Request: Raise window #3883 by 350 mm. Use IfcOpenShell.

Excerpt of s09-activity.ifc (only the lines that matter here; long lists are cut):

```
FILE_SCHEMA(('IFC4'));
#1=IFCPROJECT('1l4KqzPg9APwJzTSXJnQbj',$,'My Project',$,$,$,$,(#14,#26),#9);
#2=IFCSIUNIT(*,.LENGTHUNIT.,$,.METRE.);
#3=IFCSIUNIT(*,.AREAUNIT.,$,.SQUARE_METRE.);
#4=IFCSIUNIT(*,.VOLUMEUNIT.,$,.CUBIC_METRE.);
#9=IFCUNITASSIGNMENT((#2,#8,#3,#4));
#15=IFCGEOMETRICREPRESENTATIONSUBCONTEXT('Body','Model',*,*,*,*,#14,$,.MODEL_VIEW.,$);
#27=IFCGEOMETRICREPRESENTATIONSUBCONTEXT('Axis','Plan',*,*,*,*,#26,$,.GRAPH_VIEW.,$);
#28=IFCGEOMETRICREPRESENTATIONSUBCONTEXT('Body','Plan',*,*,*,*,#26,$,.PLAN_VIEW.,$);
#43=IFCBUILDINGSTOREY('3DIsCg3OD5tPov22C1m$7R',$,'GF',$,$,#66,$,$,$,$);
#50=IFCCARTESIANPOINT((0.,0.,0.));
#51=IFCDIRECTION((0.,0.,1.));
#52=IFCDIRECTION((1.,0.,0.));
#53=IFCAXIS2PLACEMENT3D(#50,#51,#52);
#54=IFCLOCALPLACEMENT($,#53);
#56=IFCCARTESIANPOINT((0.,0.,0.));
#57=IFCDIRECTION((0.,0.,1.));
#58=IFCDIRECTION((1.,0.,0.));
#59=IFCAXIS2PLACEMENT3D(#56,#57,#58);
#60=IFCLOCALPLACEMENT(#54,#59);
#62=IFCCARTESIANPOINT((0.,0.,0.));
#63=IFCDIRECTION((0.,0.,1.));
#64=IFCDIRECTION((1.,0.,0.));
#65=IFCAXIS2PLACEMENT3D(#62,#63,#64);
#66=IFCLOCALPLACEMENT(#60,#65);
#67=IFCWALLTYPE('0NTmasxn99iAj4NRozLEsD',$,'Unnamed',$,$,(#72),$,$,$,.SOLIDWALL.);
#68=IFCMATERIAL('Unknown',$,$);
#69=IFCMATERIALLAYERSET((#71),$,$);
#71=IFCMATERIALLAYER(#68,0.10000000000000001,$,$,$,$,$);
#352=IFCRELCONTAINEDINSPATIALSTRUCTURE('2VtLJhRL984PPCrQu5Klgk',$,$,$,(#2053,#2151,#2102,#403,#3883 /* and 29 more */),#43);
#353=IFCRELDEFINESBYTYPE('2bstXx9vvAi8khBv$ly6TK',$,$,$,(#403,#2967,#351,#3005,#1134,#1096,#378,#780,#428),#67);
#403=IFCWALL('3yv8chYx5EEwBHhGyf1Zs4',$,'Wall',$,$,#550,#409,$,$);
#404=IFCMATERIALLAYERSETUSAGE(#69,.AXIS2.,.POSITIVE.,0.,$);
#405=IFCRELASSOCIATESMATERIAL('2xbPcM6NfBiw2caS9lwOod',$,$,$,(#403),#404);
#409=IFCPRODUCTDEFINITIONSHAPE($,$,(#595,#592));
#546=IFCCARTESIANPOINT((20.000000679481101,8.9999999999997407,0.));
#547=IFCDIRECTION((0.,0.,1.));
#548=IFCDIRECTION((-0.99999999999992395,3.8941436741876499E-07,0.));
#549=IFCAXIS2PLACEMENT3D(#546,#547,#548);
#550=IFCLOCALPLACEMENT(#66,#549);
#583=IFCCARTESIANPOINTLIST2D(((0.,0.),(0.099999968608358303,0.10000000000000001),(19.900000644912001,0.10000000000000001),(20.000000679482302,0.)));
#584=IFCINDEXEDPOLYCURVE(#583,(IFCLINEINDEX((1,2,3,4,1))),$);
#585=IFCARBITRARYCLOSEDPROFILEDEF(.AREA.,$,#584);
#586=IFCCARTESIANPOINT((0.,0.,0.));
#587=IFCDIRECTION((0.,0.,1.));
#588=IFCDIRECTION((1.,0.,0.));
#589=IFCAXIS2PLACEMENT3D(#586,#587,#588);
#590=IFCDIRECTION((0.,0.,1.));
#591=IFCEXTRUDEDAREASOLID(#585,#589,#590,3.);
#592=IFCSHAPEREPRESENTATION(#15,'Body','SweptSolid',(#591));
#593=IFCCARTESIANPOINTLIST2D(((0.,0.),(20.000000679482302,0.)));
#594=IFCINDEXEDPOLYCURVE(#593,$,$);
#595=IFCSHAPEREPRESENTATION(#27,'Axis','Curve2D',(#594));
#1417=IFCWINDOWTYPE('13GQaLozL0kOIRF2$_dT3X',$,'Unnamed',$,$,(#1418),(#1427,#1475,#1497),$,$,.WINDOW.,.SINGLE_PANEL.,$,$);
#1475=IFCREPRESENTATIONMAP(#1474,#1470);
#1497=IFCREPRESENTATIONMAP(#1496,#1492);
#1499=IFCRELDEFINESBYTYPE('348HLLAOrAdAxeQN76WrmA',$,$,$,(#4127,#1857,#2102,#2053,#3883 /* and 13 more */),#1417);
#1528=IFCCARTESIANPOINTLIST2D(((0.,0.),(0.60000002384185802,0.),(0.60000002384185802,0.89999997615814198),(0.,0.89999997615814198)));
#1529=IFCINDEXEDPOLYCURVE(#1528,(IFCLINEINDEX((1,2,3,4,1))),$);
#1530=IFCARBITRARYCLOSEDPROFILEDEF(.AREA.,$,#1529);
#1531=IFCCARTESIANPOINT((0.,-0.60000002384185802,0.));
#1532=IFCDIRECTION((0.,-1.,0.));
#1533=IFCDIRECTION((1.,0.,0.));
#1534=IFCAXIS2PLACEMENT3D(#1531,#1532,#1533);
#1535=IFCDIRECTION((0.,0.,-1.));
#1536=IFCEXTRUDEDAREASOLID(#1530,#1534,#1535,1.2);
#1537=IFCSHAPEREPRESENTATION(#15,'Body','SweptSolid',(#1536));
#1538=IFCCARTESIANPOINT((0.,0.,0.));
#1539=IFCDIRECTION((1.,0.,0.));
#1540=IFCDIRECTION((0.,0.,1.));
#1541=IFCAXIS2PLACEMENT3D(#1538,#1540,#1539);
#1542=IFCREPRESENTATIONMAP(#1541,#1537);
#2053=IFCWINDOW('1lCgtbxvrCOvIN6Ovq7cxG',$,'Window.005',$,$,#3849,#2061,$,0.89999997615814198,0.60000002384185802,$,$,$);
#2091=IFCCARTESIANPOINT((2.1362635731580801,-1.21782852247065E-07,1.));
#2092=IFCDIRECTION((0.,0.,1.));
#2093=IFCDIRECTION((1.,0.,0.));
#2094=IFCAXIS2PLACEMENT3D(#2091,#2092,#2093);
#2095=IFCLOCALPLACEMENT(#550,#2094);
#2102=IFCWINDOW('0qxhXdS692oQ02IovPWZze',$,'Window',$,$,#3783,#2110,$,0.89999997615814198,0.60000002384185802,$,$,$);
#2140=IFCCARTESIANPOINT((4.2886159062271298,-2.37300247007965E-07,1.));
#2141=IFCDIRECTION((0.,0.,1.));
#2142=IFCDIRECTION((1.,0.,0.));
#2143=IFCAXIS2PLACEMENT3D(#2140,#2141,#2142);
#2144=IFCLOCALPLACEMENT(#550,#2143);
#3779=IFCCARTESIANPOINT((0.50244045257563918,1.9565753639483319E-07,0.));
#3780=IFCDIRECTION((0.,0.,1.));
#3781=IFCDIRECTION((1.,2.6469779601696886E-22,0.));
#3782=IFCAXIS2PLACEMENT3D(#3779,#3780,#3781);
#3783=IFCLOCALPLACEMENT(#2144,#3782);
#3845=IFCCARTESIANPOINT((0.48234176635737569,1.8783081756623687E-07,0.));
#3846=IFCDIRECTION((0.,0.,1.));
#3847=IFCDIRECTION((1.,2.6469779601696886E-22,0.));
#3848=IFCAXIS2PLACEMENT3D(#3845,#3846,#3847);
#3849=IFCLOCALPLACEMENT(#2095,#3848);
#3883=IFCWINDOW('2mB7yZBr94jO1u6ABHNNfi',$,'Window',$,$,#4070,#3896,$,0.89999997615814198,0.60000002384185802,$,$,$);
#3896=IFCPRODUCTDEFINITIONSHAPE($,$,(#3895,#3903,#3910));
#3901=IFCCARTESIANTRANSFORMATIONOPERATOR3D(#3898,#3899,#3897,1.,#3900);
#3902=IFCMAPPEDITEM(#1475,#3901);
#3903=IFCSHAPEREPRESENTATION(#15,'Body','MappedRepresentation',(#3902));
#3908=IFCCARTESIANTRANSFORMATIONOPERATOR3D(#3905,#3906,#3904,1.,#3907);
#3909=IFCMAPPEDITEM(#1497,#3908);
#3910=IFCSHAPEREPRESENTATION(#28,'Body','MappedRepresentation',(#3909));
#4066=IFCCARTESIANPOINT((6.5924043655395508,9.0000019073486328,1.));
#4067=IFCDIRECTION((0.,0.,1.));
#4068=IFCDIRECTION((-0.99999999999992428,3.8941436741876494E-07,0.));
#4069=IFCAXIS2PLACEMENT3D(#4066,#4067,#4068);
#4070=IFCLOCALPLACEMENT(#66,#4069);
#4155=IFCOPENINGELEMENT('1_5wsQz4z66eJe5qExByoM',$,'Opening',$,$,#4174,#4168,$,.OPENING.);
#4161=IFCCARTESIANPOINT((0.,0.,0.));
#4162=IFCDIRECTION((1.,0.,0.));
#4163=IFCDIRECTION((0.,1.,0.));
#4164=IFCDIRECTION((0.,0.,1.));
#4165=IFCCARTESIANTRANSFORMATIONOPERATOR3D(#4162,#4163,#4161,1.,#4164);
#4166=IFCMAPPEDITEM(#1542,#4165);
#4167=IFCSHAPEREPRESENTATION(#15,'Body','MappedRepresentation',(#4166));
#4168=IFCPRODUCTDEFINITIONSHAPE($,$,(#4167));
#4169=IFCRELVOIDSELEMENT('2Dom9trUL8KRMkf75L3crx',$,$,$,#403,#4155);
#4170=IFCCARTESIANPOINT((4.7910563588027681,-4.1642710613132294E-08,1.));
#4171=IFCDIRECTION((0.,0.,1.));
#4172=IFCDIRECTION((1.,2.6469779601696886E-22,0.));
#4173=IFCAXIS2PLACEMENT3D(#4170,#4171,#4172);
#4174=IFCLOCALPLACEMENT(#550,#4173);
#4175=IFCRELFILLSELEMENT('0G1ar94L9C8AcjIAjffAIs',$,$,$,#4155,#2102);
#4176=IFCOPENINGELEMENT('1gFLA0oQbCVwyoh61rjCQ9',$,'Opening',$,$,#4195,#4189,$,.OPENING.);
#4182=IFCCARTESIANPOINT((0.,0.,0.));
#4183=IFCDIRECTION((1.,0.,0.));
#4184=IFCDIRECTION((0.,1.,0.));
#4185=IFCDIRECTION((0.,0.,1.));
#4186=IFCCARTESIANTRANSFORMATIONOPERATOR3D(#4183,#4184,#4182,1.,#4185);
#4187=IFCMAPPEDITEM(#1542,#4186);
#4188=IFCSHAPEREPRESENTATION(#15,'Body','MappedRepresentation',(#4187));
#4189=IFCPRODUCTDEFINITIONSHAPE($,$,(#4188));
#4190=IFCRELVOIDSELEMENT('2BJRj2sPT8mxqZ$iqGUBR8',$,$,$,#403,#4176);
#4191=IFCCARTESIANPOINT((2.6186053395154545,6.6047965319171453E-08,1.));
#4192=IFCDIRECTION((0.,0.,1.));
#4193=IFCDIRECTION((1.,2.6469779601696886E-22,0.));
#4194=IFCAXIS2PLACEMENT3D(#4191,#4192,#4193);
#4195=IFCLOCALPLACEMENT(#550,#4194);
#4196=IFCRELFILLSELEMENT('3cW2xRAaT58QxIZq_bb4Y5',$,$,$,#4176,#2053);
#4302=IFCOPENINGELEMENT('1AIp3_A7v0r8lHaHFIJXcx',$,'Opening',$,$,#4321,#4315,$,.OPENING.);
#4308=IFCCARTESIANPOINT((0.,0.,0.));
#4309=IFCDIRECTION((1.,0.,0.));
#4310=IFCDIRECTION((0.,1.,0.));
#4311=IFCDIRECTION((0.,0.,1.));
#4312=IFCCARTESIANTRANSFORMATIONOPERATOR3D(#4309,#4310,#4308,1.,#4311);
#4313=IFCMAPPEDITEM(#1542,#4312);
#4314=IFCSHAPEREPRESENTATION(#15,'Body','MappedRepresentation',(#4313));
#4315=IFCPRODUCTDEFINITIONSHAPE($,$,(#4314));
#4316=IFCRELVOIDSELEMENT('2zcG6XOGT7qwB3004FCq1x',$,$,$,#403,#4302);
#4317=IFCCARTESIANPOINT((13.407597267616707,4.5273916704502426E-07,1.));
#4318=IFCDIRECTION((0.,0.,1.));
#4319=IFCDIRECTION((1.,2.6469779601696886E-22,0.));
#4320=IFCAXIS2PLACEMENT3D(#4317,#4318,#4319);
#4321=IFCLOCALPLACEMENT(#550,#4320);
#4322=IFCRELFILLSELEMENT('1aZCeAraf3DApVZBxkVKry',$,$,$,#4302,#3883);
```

```python
import numpy as np
import ifcopenshell
import ifcopenshell.api.geometry
import ifcopenshell.util.placement
import ifcopenshell.util.unit

model = ifcopenshell.open("s09-activity.ifc")
unit_scale = ifcopenshell.util.unit.calculate_unit_scale(model)

window = model.by_guid("2mB7yZBr94jO1u6ABHNNfi")
opening = window.FillsVoids[0].RelatingOpeningElement
dz = 0.35 / unit_scale

shift = np.array([0.0, 0.0, dz])
# The window is not placed relative to its opening, so move both.
for product in (opening, window):
    matrix = ifcopenshell.util.placement.get_local_placement(product.ObjectPlacement)
    matrix[:3, 3] += shift
    ifcopenshell.api.geometry.edit_object_placement(model, product=product, matrix=matrix, is_si=False)

print(f"moved by {dz * unit_scale:+.3f} m")

model.write("s09-activity_updated.ifc")
```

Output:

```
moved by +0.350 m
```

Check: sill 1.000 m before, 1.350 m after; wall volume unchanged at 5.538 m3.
